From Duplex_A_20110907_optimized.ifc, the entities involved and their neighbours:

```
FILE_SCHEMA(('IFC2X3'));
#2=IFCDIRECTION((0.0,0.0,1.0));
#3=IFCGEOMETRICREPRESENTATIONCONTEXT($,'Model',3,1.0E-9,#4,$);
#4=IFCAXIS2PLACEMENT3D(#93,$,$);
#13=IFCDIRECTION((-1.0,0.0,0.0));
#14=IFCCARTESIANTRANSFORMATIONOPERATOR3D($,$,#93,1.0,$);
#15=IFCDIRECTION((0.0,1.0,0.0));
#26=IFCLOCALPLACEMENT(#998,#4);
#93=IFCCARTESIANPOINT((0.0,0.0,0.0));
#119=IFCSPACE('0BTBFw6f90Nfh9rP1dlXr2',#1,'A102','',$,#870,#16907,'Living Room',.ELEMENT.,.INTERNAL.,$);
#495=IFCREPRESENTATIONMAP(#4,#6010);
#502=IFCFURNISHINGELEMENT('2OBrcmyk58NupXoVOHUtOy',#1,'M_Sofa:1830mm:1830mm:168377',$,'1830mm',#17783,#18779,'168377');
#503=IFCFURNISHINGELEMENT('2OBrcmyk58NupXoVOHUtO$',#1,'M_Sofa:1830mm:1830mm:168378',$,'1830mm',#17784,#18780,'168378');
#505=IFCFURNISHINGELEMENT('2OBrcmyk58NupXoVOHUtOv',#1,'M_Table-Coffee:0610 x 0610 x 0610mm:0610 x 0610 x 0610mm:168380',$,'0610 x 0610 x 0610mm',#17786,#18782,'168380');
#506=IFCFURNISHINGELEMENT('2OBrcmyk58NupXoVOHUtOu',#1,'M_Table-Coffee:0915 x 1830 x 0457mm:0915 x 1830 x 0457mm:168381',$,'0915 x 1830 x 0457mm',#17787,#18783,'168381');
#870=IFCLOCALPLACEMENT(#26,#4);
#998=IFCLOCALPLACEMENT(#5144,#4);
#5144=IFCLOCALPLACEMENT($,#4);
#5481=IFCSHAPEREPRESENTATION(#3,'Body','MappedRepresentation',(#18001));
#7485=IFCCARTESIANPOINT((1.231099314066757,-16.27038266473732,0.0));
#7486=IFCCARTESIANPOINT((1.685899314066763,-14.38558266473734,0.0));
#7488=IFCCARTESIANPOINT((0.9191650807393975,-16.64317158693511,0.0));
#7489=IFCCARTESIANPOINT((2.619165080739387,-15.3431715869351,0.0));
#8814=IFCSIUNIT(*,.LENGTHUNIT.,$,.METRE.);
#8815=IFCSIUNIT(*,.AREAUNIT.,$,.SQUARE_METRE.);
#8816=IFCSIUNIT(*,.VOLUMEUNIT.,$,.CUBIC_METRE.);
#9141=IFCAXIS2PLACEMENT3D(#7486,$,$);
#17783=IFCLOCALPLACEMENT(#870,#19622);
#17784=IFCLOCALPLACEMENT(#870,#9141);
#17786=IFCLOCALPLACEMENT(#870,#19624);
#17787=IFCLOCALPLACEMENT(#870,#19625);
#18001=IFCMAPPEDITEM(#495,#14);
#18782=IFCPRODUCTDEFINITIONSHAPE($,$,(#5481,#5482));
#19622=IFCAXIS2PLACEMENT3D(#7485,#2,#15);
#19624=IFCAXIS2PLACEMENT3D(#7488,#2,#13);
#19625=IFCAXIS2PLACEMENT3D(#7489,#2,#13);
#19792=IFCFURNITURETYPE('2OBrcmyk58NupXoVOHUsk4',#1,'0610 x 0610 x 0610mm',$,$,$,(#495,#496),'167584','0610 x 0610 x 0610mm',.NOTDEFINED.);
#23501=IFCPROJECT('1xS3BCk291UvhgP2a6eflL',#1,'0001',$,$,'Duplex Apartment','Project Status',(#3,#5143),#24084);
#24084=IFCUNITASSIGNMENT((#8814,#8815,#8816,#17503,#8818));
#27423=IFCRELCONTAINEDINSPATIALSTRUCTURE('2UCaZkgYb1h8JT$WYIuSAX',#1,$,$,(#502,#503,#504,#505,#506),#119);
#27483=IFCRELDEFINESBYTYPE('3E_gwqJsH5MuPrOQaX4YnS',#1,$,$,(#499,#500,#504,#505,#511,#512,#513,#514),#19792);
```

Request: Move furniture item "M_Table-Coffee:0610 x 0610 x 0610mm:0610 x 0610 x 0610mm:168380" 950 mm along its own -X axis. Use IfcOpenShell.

```python
import ifcopenshell
import ifcopenshell.api.geometry
import ifcopenshell.util.placement
import ifcopenshell.util.unit

model = ifcopenshell.open("Duplex_A_20110907_optimized.ifc")
unit_scale = ifcopenshell.util.unit.calculate_unit_scale(model)

item = model.by_guid("2OBrcmyk58NupXoVOHUtOv")
matrix = ifcopenshell.util.placement.get_local_placement(item.ObjectPlacement)
matrix[:3, 3] -= matrix[:3, 0] * 0.95 / unit_scale
ifcopenshell.api.geometry.edit_object_placement(model, product=item, matrix=matrix, is_si=False)

print(ifcopenshell.util.placement.get_local_placement(item.ObjectPlacement).round(3) + 0.0)

model.write("Duplex_A_20110907_optimized_updated.ifc")
```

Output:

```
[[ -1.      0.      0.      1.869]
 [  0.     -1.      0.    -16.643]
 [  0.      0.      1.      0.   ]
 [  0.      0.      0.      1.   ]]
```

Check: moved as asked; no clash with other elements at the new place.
